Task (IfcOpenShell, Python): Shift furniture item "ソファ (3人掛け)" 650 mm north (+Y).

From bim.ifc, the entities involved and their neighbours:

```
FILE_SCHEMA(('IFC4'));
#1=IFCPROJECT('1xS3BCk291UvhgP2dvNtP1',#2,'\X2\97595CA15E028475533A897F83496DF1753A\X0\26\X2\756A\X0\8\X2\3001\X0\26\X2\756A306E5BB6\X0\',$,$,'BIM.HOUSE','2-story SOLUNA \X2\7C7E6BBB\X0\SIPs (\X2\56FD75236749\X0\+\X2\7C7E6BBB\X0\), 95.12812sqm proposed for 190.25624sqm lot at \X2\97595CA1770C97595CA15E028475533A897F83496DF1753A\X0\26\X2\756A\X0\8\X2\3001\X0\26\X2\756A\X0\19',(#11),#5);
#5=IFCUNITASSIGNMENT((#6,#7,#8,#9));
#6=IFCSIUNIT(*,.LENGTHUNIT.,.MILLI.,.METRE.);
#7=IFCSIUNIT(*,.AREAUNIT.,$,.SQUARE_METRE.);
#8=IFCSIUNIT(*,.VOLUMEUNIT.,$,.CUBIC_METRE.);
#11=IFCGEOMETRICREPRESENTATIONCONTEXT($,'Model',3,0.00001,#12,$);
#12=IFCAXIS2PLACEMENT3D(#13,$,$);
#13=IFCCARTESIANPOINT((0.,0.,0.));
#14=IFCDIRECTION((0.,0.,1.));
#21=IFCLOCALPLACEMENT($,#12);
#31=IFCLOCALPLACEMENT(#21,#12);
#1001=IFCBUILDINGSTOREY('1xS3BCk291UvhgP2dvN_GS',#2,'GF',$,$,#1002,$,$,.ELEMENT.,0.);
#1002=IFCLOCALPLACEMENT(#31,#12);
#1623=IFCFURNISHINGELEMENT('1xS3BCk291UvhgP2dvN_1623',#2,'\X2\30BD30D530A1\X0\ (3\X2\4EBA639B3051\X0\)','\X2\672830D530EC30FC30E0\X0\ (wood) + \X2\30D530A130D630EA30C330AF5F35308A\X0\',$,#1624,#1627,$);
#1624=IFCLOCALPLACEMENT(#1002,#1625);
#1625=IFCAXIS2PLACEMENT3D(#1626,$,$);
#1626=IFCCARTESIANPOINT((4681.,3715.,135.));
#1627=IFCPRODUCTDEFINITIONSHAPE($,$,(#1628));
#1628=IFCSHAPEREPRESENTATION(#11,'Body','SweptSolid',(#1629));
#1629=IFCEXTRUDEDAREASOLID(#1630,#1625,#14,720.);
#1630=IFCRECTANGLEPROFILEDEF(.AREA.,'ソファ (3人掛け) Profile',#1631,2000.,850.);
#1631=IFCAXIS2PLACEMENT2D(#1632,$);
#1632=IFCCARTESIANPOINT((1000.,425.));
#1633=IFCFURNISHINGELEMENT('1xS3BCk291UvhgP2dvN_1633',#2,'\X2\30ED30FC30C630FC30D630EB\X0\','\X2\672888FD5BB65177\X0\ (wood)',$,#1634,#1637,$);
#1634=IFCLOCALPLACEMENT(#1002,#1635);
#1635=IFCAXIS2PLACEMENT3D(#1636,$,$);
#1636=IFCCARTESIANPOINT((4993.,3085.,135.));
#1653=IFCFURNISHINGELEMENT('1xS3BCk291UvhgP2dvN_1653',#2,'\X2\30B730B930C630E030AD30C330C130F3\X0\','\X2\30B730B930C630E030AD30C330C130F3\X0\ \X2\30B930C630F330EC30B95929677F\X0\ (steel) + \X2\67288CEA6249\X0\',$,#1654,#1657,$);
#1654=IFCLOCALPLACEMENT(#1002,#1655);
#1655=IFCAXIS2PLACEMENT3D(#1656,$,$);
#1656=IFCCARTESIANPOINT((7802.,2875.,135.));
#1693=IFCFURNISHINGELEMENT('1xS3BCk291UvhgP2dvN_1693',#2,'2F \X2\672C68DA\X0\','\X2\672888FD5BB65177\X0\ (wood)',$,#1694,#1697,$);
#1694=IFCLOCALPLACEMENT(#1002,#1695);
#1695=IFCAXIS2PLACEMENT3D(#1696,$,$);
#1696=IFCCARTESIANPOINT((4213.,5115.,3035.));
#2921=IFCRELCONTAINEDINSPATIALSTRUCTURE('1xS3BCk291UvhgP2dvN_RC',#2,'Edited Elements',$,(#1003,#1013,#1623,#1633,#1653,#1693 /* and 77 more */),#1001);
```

```python
import ifcopenshell
import ifcopenshell.api.geometry
import ifcopenshell.util.placement
import ifcopenshell.util.unit

model = ifcopenshell.open("bim.ifc")
unit_scale = ifcopenshell.util.unit.calculate_unit_scale(model)

item = model.by_id(1623)
matrix = ifcopenshell.util.placement.get_local_placement(item.ObjectPlacement)
matrix[1, 3] += 0.65 / unit_scale
ifcopenshell.api.geometry.edit_object_placement(model, product=item, matrix=matrix, is_si=False)

print(ifcopenshell.util.placement.get_local_placement(item.ObjectPlacement).round(3) + 0.0)

model.write("bim_rev.ifc")
```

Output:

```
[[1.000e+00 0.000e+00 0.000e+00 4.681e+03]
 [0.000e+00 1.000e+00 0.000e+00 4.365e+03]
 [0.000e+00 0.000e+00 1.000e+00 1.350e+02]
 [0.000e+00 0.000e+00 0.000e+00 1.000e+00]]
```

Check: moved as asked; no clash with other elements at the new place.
